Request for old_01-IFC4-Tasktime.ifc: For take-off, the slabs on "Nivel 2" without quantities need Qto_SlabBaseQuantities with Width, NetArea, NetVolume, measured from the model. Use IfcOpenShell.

First a look at what the model holds.

```python
import ifcopenshell
import ifcopenshell.util.element
import ifcopenshell.util.unit

model = ifcopenshell.open("old_01-IFC4-Tasktime.ifc")
print(model.schema)
for unit_type in ("LENGTHUNIT", "AREAUNIT", "VOLUMEUNIT"):
    print(unit_type, ifcopenshell.util.unit.calculate_unit_scale(model, unit_type))
storey = next(s for s in model.by_type("IfcBuildingStorey") if s.Name == "Nivel 2")
slabs = [e for e in ifcopenshell.util.element.get_decomposition(storey) if e.is_a("IfcSlab")]
for e in sorted(slabs, key=lambda e: e.id()):
    print(e.id(), e.is_a(), e.Name, list(ifcopenshell.util.element.get_psets(e, qtos_only=True)), sep=" | ")
```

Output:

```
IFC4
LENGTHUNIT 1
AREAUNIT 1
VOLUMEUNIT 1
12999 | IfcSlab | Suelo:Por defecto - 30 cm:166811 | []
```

```python
import ifcopenshell
import ifcopenshell.api.pset
import ifcopenshell.geom
import ifcopenshell.util.element
import ifcopenshell.util.shape
import ifcopenshell.util.unit

model = ifcopenshell.open("old_01-IFC4-Tasktime.ifc")
unit_scale = ifcopenshell.util.unit.calculate_unit_scale(model)
area_scale = ifcopenshell.util.unit.calculate_unit_scale(model, "AREAUNIT")
volume_scale = ifcopenshell.util.unit.calculate_unit_scale(model, "VOLUMEUNIT")
settings = ifcopenshell.geom.settings()

storey = next(s for s in model.by_type("IfcBuildingStorey") if s.Name == "Nivel 2")
slabs = [e for e in ifcopenshell.util.element.get_decomposition(storey) if e.is_a("IfcSlab")]

for e in sorted(slabs, key=lambda e: e.id()):
    if ifcopenshell.util.element.get_psets(e, qtos_only=True, should_inherit=False):
        continue
    # Geometry comes back in metres, in the element's own axes.
    shape = ifcopenshell.geom.create_shape(settings, e)
    values = {
        "Width": ifcopenshell.util.shape.get_z(shape.geometry) / unit_scale,
        "NetArea": ifcopenshell.util.shape.get_footprint_area(shape.geometry) / area_scale,
        "NetVolume": ifcopenshell.util.shape.get_volume(shape.geometry) / volume_scale,
    }
    qto = ifcopenshell.api.pset.add_qto(model, product=e, name="Qto_SlabBaseQuantities")
    ifcopenshell.api.pset.edit_qto(model, qto=qto, properties=values)
    print(e.id(), {k: round(v, 3) for k, v in values.items()})

model.write("old_01-IFC4-Tasktime-out.ifc")
```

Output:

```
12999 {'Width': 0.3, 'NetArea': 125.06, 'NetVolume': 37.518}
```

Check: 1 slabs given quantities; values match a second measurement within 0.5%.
